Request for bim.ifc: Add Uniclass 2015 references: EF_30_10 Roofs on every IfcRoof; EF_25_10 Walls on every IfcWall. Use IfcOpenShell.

First a look at what the model holds.

```python
import ifcopenshell

model = ifcopenshell.open("bim.ifc")
print(model.schema)
print("classifications:", [c.Name for c in model.by_type("IfcClassification")])
for ifc_class in ("IfcDoor", "IfcRoof", "IfcStair", "IfcWall", "IfcWindow"):
    print(ifc_class, len(model.by_type(ifc_class)))
```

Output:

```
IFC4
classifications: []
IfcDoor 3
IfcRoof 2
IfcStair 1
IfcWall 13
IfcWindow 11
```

```python
import ifcopenshell
import ifcopenshell.api.classification

model = ifcopenshell.open("bim.ifc")

system = ifcopenshell.api.classification.add_classification(model, classification="Uniclass 2015")

codes = {
    "IfcRoof": ("EF_30_10", "Roofs"),
    "IfcWall": ("EF_25_10", "Walls"),
}
for ifc_class, (code, name) in codes.items():
    products = model.by_type(ifc_class)
    ifcopenshell.api.classification.add_reference(
        model, products=products, classification=system, identification=code, name=name
    )
    print(code, len(products))

model.write("bim_updated.ifc")
```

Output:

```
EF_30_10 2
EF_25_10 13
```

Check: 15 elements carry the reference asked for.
